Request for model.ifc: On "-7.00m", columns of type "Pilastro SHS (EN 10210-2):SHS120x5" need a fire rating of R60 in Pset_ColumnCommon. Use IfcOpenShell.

First a look at what the model holds.

```python
import ifcopenshell
import ifcopenshell.util.element

model = ifcopenshell.open("model.ifc")
print(model.schema)
storey = next(s for s in model.by_type("IfcBuildingStorey") if s.Name == "-7.00m")
columns = [e for e in ifcopenshell.util.element.get_decomposition(storey) if e.is_a("IfcColumn")]
seen = {}
for e in columns:
    element_type = ifcopenshell.util.element.get_type(e)
    key = (element_type.Name if element_type != e and element_type else None, ifcopenshell.util.element.get_pset(e, "Pset_ColumnCommon", "FireRating"))
    seen[key] = seen.get(key, 0) + 1
for (name, value), count in sorted(seen.items(), key=str):
    print(count, "x", name, "|", value)
```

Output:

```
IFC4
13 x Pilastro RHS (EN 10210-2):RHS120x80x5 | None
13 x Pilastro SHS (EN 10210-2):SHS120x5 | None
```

```python
import ifcopenshell
import ifcopenshell.api.pset
import ifcopenshell.util.element

model = ifcopenshell.open("model.ifc")

storey = next(s for s in model.by_type("IfcBuildingStorey") if s.Name == "-7.00m")
columns = [e for e in ifcopenshell.util.element.get_decomposition(storey) if e.is_a("IfcColumn")]

count = 0
for e in columns:
    element_type = ifcopenshell.util.element.get_type(e)
    if element_type in (None, e) or element_type.Name != "Pilastro SHS (EN 10210-2):SHS120x5":
        continue
    # add_pset returns the element's existing set when there is one.
    pset = ifcopenshell.api.pset.add_pset(model, product=e, name="Pset_ColumnCommon")
    ifcopenshell.api.pset.edit_pset(model, pset=pset, properties={"FireRating": "R60"})
    count += 1

print(count, "columns updated")

model.write("model_rev.ifc")
```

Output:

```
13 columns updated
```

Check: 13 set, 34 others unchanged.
